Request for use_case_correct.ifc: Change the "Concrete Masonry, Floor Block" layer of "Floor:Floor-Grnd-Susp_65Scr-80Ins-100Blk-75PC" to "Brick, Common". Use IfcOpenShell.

First a look at what the model holds.

```python
import ifcopenshell
import ifcopenshell.util.element

model = ifcopenshell.open("use_case_correct.ifc")
print(model.schema)
for layer_set in model.by_type("IfcMaterialLayerSet"):
    if layer_set.LayerSetName == "Floor:Floor-Grnd-Susp_65Scr-80Ins-100Blk-75PC":
        for layer in layer_set.MaterialLayers:
            print(layer.id(), layer.Material and layer.Material.Name, layer.LayerThickness, sep=" | ")
        print(len(ifcopenshell.util.element.get_elements_by_material(model, layer_set)), "elements and types use it")
print(sorted(m.Name for m in model.by_type("IfcMaterial") if m.Name)[:60])
```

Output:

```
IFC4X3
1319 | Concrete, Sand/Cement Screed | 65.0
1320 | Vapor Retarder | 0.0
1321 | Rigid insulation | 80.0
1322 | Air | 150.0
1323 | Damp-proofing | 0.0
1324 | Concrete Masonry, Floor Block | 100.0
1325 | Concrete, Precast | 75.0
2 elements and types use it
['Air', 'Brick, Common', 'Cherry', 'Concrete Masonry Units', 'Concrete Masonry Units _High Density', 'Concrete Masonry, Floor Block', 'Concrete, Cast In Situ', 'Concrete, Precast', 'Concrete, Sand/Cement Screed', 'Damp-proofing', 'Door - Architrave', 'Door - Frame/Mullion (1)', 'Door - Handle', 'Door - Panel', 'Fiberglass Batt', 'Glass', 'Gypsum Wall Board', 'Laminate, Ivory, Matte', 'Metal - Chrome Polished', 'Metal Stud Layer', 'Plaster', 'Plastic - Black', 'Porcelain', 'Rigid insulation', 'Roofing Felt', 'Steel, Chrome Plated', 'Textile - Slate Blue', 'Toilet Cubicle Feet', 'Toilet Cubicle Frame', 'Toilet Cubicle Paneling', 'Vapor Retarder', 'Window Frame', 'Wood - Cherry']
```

```python
import ifcopenshell
import ifcopenshell.api.material

model = ifcopenshell.open("use_case_correct.ifc")

layer_set = next(s for s in model.by_type("IfcMaterialLayerSet") if s.LayerSetName == "Floor:Floor-Grnd-Susp_65Scr-80Ins-100Blk-75PC")
layer = next(l for l in layer_set.MaterialLayers if l.Material and l.Material.Name == "Concrete Masonry, Floor Block")
material = next(m for m in model.by_type("IfcMaterial") if m.Name == "Brick, Common")

# Point this one layer at the other material; renaming the old one would change it everywhere.
ifcopenshell.api.material.edit_layer(model, layer=layer, attributes={"Name": material.Name}, material=material)

print([l.Material.Name if l.Material else None for l in layer_set.MaterialLayers])

model.write("use_case_correct-out.ifc")
```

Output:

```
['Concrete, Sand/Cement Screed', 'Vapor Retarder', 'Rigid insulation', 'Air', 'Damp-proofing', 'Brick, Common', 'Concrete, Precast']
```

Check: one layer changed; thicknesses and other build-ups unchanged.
